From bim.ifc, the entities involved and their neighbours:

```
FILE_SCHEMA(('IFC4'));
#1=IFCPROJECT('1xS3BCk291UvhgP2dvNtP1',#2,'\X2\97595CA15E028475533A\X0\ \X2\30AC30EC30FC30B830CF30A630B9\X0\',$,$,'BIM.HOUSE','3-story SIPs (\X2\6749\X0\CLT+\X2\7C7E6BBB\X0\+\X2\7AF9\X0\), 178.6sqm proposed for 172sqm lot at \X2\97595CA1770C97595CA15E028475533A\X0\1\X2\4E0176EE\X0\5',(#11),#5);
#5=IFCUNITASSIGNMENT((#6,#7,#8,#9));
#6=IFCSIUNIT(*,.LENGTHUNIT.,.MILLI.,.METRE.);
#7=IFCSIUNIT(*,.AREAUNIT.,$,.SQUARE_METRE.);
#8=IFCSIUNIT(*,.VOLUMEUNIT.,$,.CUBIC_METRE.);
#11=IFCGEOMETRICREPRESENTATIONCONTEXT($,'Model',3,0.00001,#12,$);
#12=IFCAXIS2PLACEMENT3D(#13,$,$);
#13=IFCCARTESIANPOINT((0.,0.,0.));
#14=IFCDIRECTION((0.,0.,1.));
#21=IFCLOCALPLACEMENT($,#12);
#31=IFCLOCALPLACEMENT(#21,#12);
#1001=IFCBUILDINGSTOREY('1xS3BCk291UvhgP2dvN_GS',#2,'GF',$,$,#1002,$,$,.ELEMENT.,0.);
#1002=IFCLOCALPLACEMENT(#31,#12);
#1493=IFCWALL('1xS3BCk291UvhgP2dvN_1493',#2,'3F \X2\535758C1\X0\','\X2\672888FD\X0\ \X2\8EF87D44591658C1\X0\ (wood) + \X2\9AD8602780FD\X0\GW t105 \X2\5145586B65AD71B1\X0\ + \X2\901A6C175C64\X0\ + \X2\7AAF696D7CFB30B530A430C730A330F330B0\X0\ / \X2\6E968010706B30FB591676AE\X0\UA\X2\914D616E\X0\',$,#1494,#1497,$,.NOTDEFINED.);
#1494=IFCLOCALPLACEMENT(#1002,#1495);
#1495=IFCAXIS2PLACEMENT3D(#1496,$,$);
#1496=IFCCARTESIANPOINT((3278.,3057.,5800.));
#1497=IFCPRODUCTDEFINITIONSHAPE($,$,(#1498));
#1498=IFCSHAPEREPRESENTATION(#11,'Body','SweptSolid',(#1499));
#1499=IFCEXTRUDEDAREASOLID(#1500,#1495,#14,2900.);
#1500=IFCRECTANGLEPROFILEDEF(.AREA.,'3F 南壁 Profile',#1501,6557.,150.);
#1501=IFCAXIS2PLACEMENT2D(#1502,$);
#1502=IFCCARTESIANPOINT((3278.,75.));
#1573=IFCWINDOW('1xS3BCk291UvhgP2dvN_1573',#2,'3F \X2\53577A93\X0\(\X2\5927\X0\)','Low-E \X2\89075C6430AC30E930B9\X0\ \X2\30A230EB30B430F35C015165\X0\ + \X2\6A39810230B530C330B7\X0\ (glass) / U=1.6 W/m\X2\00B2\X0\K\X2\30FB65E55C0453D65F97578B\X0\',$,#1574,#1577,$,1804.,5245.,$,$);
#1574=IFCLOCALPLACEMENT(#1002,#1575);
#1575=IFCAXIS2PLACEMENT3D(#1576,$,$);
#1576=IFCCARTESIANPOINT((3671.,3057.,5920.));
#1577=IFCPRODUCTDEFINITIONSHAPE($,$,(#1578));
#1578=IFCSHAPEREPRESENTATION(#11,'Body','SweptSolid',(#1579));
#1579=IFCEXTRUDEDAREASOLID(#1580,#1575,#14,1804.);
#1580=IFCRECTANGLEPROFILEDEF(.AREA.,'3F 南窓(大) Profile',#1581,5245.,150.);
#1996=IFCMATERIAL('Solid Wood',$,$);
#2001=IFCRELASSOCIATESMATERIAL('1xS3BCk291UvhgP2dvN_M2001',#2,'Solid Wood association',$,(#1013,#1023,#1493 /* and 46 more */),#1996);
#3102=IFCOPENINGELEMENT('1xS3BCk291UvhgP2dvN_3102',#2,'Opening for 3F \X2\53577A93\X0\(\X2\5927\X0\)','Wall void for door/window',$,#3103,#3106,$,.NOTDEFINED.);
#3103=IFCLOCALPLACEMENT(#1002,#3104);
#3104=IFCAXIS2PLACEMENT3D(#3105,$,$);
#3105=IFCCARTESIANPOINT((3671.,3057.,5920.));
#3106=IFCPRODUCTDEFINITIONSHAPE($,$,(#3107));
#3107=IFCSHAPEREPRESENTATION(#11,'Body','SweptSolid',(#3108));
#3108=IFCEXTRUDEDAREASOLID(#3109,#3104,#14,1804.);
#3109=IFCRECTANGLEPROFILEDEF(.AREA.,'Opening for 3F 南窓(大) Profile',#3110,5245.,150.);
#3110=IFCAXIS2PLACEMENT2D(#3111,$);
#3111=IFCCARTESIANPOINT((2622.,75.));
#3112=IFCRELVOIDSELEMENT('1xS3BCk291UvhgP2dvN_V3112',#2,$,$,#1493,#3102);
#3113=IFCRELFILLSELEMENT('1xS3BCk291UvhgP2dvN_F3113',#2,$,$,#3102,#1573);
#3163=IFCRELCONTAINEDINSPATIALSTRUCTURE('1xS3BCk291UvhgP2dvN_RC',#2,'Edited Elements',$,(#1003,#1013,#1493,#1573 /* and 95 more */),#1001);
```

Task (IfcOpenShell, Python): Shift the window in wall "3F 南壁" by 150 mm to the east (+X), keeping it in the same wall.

```python
import ifcopenshell
import ifcopenshell.api.geometry
import ifcopenshell.util.placement
import ifcopenshell.util.unit

model = ifcopenshell.open("bim.ifc")
unit_scale = ifcopenshell.util.unit.calculate_unit_scale(model)

window = model.by_guid("1xS3BCk291UvhgP2dvN_1573")
opening = window.FillsVoids[0].RelatingOpeningElement
wall = opening.VoidsElements[0].RelatingBuildingElement

wall_matrix = ifcopenshell.util.placement.get_local_placement(wall.ObjectPlacement)
shift = wall_matrix[:3, 0] * 0.15 / unit_scale
before = ifcopenshell.util.placement.get_local_placement(window.ObjectPlacement)[:3, 3].copy()

# The window is not placed relative to its opening, so move both.
for product in (opening, window):
    matrix = ifcopenshell.util.placement.get_local_placement(product.ObjectPlacement)
    matrix[:3, 3] += shift
    ifcopenshell.api.geometry.edit_object_placement(model, product=product, matrix=matrix, is_si=False)

after = ifcopenshell.util.placement.get_local_placement(window.ObjectPlacement)[:3, 3]
print("window moved by", (after - before).round(3) + 0.0)

model.write("bim-out.ifc")
```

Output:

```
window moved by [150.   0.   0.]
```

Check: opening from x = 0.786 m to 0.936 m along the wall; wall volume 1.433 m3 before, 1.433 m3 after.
